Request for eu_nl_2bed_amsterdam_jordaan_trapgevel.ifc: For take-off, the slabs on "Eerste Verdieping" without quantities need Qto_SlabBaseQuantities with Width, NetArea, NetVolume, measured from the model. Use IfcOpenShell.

First a look at what the model holds.

```python
import ifcopenshell
import ifcopenshell.util.element
import ifcopenshell.util.unit

model = ifcopenshell.open("eu_nl_2bed_amsterdam_jordaan_trapgevel.ifc")
print(model.schema)
for unit_type in ("LENGTHUNIT", "AREAUNIT", "VOLUMEUNIT"):
    print(unit_type, ifcopenshell.util.unit.calculate_unit_scale(model, unit_type))
storey = next(s for s in model.by_type("IfcBuildingStorey") if s.Name == "Eerste Verdieping")
slabs = [e for e in ifcopenshell.util.element.get_decomposition(storey) if e.is_a("IfcSlab")]
for e in sorted(slabs, key=lambda e: e.id()):
    print(e.id(), e.is_a(), e.Name, list(ifcopenshell.util.element.get_psets(e, qtos_only=True)), sep=" | ")
```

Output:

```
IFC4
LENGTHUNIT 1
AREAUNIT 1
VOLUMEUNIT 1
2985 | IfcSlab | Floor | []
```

```python
import ifcopenshell
import ifcopenshell.api.pset
import ifcopenshell.geom
import ifcopenshell.util.element
import ifcopenshell.util.shape
import ifcopenshell.util.unit

model = ifcopenshell.open("eu_nl_2bed_amsterdam_jordaan_trapgevel.ifc")
unit_scale = ifcopenshell.util.unit.calculate_unit_scale(model)
area_scale = ifcopenshell.util.unit.calculate_unit_scale(model, "AREAUNIT")
volume_scale = ifcopenshell.util.unit.calculate_unit_scale(model, "VOLUMEUNIT")
settings = ifcopenshell.geom.settings()

storey = next(s for s in model.by_type("IfcBuildingStorey") if s.Name == "Eerste Verdieping")
slabs = [e for e in ifcopenshell.util.element.get_decomposition(storey) if e.is_a("IfcSlab")]

for e in sorted(slabs, key=lambda e: e.id()):
    if ifcopenshell.util.element.get_psets(e, qtos_only=True, should_inherit=False):
        continue
    # Geometry comes back in metres, in the element's own axes.
    shape = ifcopenshell.geom.create_shape(settings, e)
    values = {
        "Width": ifcopenshell.util.shape.get_z(shape.geometry) / unit_scale,
        "NetArea": ifcopenshell.util.shape.get_footprint_area(shape.geometry) / area_scale,
        "NetVolume": ifcopenshell.util.shape.get_volume(shape.geometry) / volume_scale,
    }
    qto = ifcopenshell.api.pset.add_qto(model, product=e, name="Qto_SlabBaseQuantities")
    ifcopenshell.api.pset.edit_qto(model, qto=qto, properties=values)
    print(e.id(), {k: round(v, 3) for k, v in values.items()})

model.write("eu_nl_2bed_amsterdam_jordaan_trapgevel_v2.ifc")
```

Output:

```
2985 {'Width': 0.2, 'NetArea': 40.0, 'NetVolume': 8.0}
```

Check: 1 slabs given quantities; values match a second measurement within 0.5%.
